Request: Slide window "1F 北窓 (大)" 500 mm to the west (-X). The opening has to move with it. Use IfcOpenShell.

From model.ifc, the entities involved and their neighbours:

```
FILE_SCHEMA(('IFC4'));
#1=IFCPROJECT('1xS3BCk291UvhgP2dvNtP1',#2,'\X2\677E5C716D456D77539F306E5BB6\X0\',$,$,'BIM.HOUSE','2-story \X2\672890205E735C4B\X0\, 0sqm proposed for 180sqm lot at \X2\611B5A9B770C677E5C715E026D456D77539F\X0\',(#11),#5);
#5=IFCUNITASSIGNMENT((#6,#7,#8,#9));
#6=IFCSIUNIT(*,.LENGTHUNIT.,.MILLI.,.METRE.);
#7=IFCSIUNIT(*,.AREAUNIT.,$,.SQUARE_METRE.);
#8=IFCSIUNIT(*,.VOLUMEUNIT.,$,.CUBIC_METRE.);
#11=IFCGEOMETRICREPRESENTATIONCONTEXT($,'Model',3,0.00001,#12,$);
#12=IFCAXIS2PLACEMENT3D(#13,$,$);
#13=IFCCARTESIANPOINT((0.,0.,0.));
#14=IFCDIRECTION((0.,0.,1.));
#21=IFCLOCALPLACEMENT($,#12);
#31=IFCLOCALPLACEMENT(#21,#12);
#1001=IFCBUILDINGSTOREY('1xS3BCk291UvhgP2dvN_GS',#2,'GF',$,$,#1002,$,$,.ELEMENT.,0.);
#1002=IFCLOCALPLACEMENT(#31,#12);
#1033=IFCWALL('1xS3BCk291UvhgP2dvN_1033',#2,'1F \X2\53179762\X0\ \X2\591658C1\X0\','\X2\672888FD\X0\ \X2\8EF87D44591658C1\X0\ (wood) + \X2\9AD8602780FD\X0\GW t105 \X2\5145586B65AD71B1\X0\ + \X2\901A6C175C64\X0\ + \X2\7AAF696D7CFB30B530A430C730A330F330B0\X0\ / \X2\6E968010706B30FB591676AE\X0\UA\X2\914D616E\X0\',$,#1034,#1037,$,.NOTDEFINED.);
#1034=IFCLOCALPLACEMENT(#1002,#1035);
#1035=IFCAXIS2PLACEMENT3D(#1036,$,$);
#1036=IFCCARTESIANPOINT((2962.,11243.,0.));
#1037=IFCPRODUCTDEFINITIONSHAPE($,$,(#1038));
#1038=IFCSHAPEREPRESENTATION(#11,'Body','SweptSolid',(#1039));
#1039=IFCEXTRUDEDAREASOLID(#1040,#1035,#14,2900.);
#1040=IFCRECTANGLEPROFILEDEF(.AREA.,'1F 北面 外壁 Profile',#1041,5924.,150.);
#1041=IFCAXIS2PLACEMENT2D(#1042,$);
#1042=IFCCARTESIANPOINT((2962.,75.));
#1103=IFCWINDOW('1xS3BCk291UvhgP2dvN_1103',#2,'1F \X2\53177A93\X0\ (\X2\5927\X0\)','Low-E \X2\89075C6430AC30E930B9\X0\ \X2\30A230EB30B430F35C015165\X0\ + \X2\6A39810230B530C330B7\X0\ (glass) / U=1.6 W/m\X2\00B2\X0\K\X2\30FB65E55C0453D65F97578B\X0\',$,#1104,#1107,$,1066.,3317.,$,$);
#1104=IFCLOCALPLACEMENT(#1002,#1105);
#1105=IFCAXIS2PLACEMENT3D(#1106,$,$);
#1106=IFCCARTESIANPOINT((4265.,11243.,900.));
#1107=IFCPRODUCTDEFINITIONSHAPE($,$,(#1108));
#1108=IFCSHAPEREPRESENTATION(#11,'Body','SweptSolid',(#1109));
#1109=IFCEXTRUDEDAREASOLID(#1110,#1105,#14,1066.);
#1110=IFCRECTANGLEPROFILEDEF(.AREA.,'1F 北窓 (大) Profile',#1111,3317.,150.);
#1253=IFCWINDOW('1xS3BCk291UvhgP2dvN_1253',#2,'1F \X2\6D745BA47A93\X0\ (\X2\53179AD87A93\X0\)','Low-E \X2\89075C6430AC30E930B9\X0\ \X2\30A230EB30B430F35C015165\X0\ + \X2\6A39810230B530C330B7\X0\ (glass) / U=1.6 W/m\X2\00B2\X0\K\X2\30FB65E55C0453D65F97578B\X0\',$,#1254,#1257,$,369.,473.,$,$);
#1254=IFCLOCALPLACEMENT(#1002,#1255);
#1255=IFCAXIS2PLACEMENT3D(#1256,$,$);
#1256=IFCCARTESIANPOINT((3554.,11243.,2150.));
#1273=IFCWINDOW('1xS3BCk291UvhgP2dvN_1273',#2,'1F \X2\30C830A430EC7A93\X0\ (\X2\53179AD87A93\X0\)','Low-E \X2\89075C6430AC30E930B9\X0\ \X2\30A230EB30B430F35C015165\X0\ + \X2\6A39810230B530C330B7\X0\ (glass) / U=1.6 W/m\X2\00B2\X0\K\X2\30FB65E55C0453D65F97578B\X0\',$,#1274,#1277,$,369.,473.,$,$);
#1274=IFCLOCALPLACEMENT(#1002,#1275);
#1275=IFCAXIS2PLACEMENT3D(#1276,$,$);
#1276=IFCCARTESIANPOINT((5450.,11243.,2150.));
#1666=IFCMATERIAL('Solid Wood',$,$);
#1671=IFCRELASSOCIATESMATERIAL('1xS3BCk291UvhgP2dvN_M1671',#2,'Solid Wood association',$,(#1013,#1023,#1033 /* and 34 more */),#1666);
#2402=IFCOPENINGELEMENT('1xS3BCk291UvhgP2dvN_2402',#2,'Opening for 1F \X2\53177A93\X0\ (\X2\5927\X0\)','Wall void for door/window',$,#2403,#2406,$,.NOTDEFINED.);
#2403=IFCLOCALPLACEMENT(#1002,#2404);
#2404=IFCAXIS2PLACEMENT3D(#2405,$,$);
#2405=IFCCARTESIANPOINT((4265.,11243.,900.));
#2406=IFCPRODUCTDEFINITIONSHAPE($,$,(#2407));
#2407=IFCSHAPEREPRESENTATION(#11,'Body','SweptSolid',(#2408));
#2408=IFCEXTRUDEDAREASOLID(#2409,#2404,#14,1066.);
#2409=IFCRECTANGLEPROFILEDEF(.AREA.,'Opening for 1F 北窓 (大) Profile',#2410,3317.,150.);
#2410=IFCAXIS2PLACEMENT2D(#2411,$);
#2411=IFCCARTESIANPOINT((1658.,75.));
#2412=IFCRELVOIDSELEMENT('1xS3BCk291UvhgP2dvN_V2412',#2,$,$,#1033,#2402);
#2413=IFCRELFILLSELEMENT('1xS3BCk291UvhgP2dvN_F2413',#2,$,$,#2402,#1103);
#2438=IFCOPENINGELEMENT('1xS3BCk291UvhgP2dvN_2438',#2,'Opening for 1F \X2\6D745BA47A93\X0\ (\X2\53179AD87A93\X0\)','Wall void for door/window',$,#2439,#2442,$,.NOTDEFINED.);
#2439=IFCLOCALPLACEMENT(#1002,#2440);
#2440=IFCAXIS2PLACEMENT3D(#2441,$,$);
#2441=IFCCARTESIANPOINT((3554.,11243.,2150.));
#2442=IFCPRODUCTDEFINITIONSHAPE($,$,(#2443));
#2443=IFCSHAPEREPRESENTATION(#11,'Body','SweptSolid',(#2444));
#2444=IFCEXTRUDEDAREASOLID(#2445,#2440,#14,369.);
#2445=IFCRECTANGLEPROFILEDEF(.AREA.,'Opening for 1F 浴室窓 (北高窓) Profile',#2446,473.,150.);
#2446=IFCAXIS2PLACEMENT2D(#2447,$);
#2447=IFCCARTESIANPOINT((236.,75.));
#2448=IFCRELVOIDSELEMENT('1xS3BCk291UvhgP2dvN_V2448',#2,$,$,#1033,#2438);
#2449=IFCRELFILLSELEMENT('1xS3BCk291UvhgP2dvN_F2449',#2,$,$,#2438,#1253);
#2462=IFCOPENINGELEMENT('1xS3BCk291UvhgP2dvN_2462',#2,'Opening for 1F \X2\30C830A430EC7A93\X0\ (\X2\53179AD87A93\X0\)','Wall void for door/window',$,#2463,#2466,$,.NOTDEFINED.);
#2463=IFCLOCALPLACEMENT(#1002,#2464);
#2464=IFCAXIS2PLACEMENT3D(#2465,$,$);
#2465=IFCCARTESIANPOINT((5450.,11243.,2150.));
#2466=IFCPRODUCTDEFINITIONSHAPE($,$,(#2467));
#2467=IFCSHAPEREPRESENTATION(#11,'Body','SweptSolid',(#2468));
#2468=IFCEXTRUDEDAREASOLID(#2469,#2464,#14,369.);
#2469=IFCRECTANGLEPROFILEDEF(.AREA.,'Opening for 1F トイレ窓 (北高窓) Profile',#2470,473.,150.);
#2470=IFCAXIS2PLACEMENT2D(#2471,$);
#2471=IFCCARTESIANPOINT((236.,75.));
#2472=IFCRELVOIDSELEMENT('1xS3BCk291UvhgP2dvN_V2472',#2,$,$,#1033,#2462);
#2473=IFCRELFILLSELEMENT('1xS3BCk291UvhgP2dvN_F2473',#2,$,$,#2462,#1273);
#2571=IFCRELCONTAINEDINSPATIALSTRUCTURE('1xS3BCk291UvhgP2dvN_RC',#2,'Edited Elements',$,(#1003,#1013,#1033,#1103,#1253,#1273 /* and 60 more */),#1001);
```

```python
import ifcopenshell
import ifcopenshell.api.geometry
import ifcopenshell.util.placement
import ifcopenshell.util.unit

model = ifcopenshell.open("model.ifc")
unit_scale = ifcopenshell.util.unit.calculate_unit_scale(model)

window = model.by_guid("1xS3BCk291UvhgP2dvN_1103")
opening = window.FillsVoids[0].RelatingOpeningElement
wall = opening.VoidsElements[0].RelatingBuildingElement

wall_matrix = ifcopenshell.util.placement.get_local_placement(wall.ObjectPlacement)
shift = wall_matrix[:3, 0] * -0.5 / unit_scale
before = ifcopenshell.util.placement.get_local_placement(window.ObjectPlacement)[:3, 3].copy()

# The window is not placed relative to its opening, so move both.
for product in (opening, window):
    matrix = ifcopenshell.util.placement.get_local_placement(product.ObjectPlacement)
    matrix[:3, 3] += shift
    ifcopenshell.api.geometry.edit_object_placement(model, product=product, matrix=matrix, is_si=False)

after = ifcopenshell.util.placement.get_local_placement(window.ObjectPlacement)[:3, 3]
print("window moved by", (after - before).round(3) + 0.0)

model.write("model_updated.ifc")
```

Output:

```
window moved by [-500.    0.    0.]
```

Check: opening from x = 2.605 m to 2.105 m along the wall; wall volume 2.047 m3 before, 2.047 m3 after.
